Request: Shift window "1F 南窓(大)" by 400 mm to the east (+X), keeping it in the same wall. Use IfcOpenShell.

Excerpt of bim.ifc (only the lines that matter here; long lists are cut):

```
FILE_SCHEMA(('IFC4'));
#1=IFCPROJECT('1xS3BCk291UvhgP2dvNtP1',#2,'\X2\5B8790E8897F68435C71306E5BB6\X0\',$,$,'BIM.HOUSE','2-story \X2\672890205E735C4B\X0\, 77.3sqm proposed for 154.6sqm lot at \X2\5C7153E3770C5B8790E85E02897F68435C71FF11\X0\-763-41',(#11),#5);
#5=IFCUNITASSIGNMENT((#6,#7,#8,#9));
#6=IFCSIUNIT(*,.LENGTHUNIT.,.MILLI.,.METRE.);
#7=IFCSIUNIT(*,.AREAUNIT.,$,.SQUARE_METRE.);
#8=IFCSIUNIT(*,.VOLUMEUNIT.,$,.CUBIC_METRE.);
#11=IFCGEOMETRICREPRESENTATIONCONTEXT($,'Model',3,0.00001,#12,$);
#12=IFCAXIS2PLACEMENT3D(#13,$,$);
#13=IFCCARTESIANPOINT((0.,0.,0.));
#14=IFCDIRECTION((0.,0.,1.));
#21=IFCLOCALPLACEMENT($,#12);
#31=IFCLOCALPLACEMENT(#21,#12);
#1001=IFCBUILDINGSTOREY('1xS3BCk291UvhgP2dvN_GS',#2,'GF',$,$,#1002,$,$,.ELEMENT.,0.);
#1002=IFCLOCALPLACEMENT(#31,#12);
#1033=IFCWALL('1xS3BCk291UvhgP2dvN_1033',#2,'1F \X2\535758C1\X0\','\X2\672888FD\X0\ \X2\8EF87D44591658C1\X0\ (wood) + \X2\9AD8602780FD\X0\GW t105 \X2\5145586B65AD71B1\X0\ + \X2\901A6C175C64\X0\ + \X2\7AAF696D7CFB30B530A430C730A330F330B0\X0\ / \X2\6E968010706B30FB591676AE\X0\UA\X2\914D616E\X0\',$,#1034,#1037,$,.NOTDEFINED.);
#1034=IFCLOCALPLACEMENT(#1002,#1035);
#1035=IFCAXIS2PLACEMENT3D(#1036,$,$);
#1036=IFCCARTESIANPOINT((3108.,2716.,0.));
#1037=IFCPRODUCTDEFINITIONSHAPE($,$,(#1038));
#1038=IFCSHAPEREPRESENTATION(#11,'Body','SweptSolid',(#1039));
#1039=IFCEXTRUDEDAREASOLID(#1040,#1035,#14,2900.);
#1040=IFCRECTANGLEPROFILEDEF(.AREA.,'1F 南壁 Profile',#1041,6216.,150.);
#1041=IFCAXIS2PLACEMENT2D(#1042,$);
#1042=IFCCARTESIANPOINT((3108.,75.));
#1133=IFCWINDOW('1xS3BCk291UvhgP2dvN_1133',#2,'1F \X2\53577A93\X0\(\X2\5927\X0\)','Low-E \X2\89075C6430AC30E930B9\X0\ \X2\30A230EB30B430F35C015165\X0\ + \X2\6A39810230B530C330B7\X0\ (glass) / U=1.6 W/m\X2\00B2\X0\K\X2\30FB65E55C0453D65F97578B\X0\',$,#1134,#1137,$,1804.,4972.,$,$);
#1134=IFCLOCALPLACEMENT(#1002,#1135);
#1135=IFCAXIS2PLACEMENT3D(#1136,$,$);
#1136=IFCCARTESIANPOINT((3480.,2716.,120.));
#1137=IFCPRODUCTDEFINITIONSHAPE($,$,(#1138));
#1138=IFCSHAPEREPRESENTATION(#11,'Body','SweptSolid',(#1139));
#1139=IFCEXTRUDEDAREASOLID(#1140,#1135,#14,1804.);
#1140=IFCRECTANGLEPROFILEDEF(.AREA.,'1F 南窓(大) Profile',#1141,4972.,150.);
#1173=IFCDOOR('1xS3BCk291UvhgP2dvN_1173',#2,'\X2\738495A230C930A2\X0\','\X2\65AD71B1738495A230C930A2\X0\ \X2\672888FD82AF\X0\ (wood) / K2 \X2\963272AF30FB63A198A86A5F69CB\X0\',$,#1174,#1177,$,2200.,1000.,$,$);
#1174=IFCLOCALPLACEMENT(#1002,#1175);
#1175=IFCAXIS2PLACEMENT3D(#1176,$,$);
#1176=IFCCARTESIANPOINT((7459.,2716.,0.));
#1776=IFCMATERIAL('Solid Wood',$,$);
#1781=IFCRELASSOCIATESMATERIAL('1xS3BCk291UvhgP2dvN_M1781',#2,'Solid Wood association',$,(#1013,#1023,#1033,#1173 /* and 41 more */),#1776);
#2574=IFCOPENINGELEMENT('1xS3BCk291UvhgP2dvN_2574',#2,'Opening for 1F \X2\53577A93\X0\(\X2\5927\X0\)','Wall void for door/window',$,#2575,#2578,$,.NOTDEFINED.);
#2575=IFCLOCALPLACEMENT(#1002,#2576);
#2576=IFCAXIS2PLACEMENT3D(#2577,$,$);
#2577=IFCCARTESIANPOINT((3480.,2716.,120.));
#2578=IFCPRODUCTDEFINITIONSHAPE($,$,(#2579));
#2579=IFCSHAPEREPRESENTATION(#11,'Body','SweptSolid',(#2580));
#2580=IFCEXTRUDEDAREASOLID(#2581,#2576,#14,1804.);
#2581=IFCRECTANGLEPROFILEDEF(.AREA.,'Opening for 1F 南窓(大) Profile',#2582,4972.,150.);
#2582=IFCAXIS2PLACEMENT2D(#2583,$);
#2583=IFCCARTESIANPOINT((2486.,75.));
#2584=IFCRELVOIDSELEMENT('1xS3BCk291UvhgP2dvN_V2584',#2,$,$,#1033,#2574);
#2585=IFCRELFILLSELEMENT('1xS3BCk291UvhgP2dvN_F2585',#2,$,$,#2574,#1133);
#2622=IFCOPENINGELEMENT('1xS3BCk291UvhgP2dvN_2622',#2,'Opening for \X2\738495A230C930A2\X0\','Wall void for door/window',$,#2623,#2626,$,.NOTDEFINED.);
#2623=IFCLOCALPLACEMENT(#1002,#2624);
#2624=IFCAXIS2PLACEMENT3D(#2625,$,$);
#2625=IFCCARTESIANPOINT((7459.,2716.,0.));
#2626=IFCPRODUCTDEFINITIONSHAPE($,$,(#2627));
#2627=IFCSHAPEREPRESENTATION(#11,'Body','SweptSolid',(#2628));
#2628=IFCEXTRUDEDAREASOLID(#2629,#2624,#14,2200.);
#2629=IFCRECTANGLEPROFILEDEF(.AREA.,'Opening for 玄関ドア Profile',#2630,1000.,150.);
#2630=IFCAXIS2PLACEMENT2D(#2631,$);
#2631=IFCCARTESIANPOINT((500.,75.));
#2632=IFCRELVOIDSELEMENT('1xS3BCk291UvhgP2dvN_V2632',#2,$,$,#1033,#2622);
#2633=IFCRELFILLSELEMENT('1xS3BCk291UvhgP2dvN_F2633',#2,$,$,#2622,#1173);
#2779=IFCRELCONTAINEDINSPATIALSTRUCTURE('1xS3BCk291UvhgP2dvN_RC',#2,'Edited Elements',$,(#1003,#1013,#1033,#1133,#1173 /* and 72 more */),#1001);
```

```python
import ifcopenshell
import ifcopenshell.api.geometry
import ifcopenshell.util.placement

model = ifcopenshell.open("bim.ifc")

window = model.by_id(1133)
opening = window.FillsVoids[0].RelatingOpeningElement
wall = opening.VoidsElements[0].RelatingBuildingElement

wall_matrix = ifcopenshell.util.placement.get_local_placement(wall.ObjectPlacement)
shift = wall_matrix[:3, 0] * 400.0
before = ifcopenshell.util.placement.get_local_placement(window.ObjectPlacement)[:3, 3].copy()

# The window is not placed relative to its opening, so move both.
for product in (opening, window):
    matrix = ifcopenshell.util.placement.get_local_placement(product.ObjectPlacement)
    matrix[:3, 3] += shift
    ifcopenshell.api.geometry.edit_object_placement(model, product=product, matrix=matrix, is_si=False)

after = ifcopenshell.util.placement.get_local_placement(window.ObjectPlacement)[:3, 3]
print("window moved by", (after - before).round(3) + 0.0)

model.write("bim-out.ifc")
```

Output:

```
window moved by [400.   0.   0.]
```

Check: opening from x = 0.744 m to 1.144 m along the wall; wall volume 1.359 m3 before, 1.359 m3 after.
